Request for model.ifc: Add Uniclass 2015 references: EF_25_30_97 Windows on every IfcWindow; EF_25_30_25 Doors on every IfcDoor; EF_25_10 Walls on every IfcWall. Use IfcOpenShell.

First a look at what the model holds.

```python
import ifcopenshell

model = ifcopenshell.open("model.ifc")
print(model.schema)
print("classifications:", [c.Name for c in model.by_type("IfcClassification")])
for ifc_class in ("IfcDoor", "IfcRoof", "IfcStair", "IfcWall", "IfcWindow"):
    print(ifc_class, len(model.by_type(ifc_class)))
```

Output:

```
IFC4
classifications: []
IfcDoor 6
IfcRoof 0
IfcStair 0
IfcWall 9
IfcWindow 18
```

```python
import ifcopenshell
import ifcopenshell.api.classification

model = ifcopenshell.open("model.ifc")

system = ifcopenshell.api.classification.add_classification(model, classification="Uniclass 2015")

codes = {
    "IfcWindow": ("EF_25_30_97", "Windows"),
    "IfcDoor": ("EF_25_30_25", "Doors"),
    "IfcWall": ("EF_25_10", "Walls"),
}
for ifc_class, (code, name) in codes.items():
    products = model.by_type(ifc_class)
    ifcopenshell.api.classification.add_reference(
        model, products=products, classification=system, identification=code, name=name
    )
    print(code, len(products))

model.write("model_edited.ifc")
```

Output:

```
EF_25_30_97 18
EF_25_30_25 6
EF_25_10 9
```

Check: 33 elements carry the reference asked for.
